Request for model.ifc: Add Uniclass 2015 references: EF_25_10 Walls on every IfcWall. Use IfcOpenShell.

First a look at what the model holds.

```python
import ifcopenshell

model = ifcopenshell.open("model.ifc")
print(model.schema)
print("classifications:", [c.Name for c in model.by_type("IfcClassification")])
for ifc_class in ("IfcDoor", "IfcRoof", "IfcStair", "IfcWall", "IfcWindow"):
    print(ifc_class, len(model.by_type(ifc_class)))
```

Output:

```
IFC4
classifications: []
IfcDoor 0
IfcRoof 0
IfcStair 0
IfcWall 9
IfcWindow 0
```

```python
import ifcopenshell
import ifcopenshell.api.classification

model = ifcopenshell.open("model.ifc")

system = ifcopenshell.api.classification.add_classification(model, classification="Uniclass 2015")

codes = {
    "IfcWall": ("EF_25_10", "Walls"),
}
for ifc_class, (code, name) in codes.items():
    products = model.by_type(ifc_class)
    ifcopenshell.api.classification.add_reference(
        model, products=products, classification=system, identification=code, name=name
    )
    print(code, len(products))

model.write("model_rev.ifc")
```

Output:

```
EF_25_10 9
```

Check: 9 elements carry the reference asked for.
